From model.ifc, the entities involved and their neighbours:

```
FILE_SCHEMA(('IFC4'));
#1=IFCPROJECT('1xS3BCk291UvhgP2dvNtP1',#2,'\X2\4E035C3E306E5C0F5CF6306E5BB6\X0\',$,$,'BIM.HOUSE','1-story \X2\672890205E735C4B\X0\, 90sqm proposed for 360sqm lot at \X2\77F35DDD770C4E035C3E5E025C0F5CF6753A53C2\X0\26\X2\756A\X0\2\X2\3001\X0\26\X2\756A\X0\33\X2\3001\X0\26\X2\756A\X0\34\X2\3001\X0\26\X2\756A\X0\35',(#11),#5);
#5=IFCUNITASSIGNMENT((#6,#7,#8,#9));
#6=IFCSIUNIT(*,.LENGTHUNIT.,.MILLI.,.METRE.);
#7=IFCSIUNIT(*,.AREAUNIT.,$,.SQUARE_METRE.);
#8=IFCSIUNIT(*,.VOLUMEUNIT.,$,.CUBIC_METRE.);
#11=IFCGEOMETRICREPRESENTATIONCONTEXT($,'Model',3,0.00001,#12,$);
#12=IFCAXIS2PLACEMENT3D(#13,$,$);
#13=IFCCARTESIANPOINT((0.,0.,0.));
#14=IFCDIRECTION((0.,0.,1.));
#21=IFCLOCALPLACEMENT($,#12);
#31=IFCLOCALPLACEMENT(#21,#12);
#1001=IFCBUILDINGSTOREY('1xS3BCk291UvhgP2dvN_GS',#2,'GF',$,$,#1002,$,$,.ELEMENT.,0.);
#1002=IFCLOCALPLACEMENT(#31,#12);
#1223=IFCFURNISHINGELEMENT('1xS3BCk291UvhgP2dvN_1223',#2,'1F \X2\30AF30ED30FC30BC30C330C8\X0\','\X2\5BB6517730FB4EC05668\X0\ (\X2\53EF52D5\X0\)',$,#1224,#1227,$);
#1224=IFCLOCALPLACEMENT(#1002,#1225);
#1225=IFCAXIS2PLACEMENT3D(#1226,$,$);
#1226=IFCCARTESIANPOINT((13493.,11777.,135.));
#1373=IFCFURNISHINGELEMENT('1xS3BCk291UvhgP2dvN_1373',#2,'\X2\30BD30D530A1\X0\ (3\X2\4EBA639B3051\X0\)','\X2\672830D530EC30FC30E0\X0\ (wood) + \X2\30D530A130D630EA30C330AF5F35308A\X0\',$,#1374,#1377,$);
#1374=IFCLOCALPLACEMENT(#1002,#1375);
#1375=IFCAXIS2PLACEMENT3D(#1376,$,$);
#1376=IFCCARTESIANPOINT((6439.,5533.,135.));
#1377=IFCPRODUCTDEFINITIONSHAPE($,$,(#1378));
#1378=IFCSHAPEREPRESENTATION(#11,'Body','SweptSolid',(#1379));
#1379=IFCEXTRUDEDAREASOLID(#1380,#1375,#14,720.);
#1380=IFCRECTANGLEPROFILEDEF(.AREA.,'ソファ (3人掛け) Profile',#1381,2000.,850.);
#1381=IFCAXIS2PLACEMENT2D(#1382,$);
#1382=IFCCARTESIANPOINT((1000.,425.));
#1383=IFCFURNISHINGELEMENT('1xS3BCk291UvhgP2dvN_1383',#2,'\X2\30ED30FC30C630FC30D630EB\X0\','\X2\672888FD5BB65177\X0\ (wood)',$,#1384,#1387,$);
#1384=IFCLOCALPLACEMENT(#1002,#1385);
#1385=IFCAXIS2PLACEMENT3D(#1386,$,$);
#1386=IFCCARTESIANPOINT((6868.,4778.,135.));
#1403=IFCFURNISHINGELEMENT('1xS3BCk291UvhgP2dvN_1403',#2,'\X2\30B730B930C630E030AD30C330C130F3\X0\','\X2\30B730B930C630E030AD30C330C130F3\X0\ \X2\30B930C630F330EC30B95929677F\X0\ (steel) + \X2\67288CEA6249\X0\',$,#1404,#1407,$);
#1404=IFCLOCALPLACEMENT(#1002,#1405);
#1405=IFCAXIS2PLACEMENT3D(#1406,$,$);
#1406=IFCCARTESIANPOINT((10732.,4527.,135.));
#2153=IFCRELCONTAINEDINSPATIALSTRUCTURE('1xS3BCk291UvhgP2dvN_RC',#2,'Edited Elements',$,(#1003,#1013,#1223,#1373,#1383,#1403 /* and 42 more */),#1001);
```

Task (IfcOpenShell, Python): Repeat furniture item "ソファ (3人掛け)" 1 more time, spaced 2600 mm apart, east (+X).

```python
import numpy as np
import ifcopenshell
import ifcopenshell.api.geometry
import ifcopenshell.api.root
import ifcopenshell.util.element
import ifcopenshell.util.placement

model = ifcopenshell.open("model.ifc")


def reuse_history(source, copy):
    """copy_class also copies each property set's owner history, people and application; keep the originals."""
    for rel in copy.IsDefinedBy:
        if rel.is_a("IfcRelDefinesByProperties") and (history := rel.RelatingPropertyDefinition.OwnerHistory):
            rel.RelatingPropertyDefinition.OwnerHistory = source.OwnerHistory
            ifcopenshell.util.element.remove_deep2(model, history)


source = model.by_guid("1xS3BCk291UvhgP2dvN_1373")
base = ifcopenshell.util.placement.get_local_placement(source.ObjectPlacement)
step = np.array([1.0, 0.0, 0.0]) * 2600.0

for i in range(1, 2):
    copy = ifcopenshell.api.root.copy_class(model, product=source)
    copy.Representation = ifcopenshell.util.element.copy_deep(
        model, source.Representation, exclude=["IfcGeometricRepresentationContext", "IfcRepresentationMap"]
    )
    reuse_history(source, copy)
    matrix = base.copy()
    matrix[:3, 3] += i * step
    print("added at", matrix[:3, 3].round(3) + 0.0)
    ifcopenshell.api.geometry.edit_object_placement(model, product=copy, matrix=matrix, is_si=False)

model.write("model-out.ifc")
```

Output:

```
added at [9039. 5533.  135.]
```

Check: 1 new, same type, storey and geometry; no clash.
